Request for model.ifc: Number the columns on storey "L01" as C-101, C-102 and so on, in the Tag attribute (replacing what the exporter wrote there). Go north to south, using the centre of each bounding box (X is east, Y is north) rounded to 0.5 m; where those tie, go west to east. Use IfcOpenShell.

First a look at what the model holds.

```python
import ifcopenshell
import ifcopenshell.util.element
import ifcopenshell.util.placement

model = ifcopenshell.open("model.ifc")
print(model.schema)
storey = next(s for s in model.by_type("IfcBuildingStorey") if s.Name == "L01")
columns = [e for e in ifcopenshell.util.element.get_decomposition(storey) if e.is_a("IfcColumn")]
for e in sorted(columns, key=lambda e: e.id()):
    origin = ifcopenshell.util.placement.get_local_placement(e.ObjectPlacement)[:3, 3]
    print(e.id(), e.Tag, e.Name, origin.round(2) + 0.0, sep=" | ")
```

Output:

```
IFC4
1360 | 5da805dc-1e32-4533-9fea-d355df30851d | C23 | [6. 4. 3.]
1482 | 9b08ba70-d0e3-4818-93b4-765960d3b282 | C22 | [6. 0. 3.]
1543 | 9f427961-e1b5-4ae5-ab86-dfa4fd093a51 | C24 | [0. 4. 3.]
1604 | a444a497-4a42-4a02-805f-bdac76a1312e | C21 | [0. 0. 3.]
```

```python
import ifcopenshell
import ifcopenshell.geom
import ifcopenshell.util.element
import ifcopenshell.util.shape

model = ifcopenshell.open("model.ifc")
settings = ifcopenshell.geom.settings()
settings.set("use-world-coords", True)


def centre(element):
    shape = ifcopenshell.geom.create_shape(settings, element)
    return ifcopenshell.util.shape.get_bbox_centroid(shape.geometry)


storey = next(s for s in model.by_type("IfcBuildingStorey") if s.Name == "L01")
columns = [e for e in ifcopenshell.util.element.get_decomposition(storey) if e.is_a("IfcColumn")]

# Insertion points can sit at a corner or the storey origin, so sort by the geometry (in metres).
centres = {e: centre(e) for e in columns}
columns.sort(key=lambda e: (-round(centres[e][1] / 0.5), centres[e][0]))

for i, e in enumerate(columns, start=1):
    number = f"C-1{i:02d}"
    e.Tag = number
    print(e.id(), number)

model.write("model-out.ifc")
```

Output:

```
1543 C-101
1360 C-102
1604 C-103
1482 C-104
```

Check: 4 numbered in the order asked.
